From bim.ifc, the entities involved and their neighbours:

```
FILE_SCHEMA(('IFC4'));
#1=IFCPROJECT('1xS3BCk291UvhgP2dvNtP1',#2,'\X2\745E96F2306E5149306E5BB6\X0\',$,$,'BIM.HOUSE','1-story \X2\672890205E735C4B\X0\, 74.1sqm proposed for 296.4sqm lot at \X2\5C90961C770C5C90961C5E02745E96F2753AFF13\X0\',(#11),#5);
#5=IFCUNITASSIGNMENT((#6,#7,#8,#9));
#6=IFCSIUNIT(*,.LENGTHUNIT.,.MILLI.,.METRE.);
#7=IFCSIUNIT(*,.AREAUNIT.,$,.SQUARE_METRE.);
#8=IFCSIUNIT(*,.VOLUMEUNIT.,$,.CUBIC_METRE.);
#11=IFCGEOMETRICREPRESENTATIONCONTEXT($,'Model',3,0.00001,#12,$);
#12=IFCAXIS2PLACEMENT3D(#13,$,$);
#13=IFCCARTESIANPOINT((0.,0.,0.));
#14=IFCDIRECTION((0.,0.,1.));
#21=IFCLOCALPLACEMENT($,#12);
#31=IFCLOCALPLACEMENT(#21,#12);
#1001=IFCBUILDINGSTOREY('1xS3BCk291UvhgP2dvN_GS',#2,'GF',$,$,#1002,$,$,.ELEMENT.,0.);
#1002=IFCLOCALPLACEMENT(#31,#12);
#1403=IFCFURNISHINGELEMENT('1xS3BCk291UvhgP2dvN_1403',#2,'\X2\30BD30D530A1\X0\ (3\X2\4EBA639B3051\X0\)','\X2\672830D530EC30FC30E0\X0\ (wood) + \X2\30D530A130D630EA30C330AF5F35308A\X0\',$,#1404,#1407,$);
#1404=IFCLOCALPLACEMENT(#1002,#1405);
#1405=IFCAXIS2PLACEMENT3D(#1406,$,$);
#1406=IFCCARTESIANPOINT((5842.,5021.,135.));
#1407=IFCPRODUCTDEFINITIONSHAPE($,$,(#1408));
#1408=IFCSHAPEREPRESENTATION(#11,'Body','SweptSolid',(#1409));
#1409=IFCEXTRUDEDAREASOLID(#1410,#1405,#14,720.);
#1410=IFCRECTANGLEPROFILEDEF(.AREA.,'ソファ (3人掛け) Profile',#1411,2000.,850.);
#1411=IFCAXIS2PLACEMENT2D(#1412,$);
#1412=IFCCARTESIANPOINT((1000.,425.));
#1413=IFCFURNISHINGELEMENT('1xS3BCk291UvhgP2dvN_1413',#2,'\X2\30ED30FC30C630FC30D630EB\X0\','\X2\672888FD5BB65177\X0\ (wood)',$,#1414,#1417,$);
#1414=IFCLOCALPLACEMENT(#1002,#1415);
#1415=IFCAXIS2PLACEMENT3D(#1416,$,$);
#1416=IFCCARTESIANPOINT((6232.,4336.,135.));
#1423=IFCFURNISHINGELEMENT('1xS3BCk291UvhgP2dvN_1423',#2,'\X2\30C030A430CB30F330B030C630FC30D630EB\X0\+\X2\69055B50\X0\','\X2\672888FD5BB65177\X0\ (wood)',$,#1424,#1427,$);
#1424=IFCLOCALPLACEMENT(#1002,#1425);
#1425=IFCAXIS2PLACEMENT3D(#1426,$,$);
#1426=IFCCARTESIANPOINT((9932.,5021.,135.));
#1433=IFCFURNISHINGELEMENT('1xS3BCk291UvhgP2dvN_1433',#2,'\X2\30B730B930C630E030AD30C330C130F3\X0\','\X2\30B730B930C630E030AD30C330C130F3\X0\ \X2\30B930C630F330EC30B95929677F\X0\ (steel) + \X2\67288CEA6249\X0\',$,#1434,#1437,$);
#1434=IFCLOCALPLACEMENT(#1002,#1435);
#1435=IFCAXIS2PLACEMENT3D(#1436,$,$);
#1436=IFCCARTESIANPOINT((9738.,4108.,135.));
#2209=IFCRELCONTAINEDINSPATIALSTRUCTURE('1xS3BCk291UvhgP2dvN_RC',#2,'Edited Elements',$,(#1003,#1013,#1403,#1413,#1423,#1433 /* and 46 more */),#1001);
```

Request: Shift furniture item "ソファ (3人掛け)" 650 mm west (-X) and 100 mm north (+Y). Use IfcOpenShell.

```python
import ifcopenshell
import ifcopenshell.api.geometry
import ifcopenshell.util.placement

model = ifcopenshell.open("bim.ifc")

item = model.by_id(1403)
matrix = ifcopenshell.util.placement.get_local_placement(item.ObjectPlacement)
matrix[0, 3] -= 650.0
matrix[1, 3] += 100.0
ifcopenshell.api.geometry.edit_object_placement(model, product=item, matrix=matrix, is_si=False)

print(ifcopenshell.util.placement.get_local_placement(item.ObjectPlacement).round(3) + 0.0)

model.write("bim_edited.ifc")
```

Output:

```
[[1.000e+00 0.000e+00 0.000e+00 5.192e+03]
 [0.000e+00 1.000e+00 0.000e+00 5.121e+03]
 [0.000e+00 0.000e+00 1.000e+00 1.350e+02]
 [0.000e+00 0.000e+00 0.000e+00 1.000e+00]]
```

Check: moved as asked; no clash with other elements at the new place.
